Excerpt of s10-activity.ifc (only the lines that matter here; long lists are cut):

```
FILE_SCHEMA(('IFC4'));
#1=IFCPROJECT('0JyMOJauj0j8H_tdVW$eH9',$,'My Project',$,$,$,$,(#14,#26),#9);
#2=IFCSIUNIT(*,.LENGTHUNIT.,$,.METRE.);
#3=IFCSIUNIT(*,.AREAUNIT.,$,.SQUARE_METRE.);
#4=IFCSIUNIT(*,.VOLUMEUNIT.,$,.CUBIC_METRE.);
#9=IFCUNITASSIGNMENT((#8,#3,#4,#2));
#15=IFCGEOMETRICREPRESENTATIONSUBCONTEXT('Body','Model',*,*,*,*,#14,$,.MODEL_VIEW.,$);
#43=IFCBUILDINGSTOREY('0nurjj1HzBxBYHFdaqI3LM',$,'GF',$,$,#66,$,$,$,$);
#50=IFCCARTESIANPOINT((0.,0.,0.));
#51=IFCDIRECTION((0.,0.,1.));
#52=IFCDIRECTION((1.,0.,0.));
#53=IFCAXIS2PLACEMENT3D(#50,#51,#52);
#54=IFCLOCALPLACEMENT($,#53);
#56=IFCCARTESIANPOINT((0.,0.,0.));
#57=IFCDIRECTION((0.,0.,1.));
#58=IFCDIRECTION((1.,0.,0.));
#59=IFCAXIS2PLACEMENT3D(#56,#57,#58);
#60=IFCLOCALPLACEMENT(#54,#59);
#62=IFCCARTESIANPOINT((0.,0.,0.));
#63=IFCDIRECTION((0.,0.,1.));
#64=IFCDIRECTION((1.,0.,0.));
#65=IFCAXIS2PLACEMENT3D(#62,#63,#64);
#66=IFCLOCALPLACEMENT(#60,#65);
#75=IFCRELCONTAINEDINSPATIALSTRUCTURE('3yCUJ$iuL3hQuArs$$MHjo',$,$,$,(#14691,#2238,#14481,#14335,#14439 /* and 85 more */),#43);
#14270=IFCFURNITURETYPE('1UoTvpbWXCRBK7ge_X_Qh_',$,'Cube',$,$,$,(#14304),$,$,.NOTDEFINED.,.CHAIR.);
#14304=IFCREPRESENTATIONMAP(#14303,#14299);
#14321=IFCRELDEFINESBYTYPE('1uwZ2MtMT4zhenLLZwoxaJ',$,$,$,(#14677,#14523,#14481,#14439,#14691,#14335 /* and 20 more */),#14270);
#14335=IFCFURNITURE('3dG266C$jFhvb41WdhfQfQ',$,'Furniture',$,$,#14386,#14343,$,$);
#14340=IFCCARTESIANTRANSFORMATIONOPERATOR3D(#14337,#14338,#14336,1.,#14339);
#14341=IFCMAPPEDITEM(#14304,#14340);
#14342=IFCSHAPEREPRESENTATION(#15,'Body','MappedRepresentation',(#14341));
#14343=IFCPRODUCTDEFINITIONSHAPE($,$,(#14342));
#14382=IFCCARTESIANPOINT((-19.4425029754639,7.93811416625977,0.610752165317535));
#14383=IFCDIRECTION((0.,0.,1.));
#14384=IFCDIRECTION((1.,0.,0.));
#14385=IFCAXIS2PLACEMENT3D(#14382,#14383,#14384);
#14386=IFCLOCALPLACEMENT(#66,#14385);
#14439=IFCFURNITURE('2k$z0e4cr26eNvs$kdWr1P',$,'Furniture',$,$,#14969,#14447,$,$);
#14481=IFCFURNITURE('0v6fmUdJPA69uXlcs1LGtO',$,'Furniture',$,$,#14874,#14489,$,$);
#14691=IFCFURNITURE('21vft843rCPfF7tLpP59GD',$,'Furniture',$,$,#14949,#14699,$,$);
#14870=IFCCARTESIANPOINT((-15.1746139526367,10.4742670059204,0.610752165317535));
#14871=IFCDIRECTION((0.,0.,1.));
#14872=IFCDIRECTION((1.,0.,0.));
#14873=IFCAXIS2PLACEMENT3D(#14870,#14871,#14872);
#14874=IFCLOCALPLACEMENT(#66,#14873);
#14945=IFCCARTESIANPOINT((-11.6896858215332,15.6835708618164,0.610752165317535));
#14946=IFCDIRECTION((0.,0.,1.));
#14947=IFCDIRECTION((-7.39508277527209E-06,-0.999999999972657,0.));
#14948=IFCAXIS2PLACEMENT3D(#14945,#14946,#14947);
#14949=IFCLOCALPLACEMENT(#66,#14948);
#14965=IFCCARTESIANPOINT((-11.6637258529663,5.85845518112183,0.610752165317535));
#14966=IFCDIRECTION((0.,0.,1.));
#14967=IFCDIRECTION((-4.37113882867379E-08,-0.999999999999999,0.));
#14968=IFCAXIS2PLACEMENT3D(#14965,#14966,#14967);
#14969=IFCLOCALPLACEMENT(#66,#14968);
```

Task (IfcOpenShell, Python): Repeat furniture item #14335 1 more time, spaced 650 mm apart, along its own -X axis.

```python
import ifcopenshell
import ifcopenshell.api.geometry
import ifcopenshell.api.root
import ifcopenshell.util.element
import ifcopenshell.util.placement
import ifcopenshell.util.unit

model = ifcopenshell.open("s10-activity.ifc")
unit_scale = ifcopenshell.util.unit.calculate_unit_scale(model)

source = model.by_guid("3dG266C$jFhvb41WdhfQfQ")
base = ifcopenshell.util.placement.get_local_placement(source.ObjectPlacement)
step = -base[:3, 0] * 0.65 / unit_scale

for i in range(1, 2):
    copy = ifcopenshell.api.root.copy_class(model, product=source)
    copy.Representation = ifcopenshell.util.element.copy_deep(
        model, source.Representation, exclude=["IfcGeometricRepresentationContext", "IfcRepresentationMap"]
    )
    matrix = base.copy()
    matrix[:3, 3] += i * step
    print("added at", matrix[:3, 3].round(3) + 0.0)
    ifcopenshell.api.geometry.edit_object_placement(model, product=copy, matrix=matrix, is_si=False)

model.write("s10-activity_v2.ifc")
```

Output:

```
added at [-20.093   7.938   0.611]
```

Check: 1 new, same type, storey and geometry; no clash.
